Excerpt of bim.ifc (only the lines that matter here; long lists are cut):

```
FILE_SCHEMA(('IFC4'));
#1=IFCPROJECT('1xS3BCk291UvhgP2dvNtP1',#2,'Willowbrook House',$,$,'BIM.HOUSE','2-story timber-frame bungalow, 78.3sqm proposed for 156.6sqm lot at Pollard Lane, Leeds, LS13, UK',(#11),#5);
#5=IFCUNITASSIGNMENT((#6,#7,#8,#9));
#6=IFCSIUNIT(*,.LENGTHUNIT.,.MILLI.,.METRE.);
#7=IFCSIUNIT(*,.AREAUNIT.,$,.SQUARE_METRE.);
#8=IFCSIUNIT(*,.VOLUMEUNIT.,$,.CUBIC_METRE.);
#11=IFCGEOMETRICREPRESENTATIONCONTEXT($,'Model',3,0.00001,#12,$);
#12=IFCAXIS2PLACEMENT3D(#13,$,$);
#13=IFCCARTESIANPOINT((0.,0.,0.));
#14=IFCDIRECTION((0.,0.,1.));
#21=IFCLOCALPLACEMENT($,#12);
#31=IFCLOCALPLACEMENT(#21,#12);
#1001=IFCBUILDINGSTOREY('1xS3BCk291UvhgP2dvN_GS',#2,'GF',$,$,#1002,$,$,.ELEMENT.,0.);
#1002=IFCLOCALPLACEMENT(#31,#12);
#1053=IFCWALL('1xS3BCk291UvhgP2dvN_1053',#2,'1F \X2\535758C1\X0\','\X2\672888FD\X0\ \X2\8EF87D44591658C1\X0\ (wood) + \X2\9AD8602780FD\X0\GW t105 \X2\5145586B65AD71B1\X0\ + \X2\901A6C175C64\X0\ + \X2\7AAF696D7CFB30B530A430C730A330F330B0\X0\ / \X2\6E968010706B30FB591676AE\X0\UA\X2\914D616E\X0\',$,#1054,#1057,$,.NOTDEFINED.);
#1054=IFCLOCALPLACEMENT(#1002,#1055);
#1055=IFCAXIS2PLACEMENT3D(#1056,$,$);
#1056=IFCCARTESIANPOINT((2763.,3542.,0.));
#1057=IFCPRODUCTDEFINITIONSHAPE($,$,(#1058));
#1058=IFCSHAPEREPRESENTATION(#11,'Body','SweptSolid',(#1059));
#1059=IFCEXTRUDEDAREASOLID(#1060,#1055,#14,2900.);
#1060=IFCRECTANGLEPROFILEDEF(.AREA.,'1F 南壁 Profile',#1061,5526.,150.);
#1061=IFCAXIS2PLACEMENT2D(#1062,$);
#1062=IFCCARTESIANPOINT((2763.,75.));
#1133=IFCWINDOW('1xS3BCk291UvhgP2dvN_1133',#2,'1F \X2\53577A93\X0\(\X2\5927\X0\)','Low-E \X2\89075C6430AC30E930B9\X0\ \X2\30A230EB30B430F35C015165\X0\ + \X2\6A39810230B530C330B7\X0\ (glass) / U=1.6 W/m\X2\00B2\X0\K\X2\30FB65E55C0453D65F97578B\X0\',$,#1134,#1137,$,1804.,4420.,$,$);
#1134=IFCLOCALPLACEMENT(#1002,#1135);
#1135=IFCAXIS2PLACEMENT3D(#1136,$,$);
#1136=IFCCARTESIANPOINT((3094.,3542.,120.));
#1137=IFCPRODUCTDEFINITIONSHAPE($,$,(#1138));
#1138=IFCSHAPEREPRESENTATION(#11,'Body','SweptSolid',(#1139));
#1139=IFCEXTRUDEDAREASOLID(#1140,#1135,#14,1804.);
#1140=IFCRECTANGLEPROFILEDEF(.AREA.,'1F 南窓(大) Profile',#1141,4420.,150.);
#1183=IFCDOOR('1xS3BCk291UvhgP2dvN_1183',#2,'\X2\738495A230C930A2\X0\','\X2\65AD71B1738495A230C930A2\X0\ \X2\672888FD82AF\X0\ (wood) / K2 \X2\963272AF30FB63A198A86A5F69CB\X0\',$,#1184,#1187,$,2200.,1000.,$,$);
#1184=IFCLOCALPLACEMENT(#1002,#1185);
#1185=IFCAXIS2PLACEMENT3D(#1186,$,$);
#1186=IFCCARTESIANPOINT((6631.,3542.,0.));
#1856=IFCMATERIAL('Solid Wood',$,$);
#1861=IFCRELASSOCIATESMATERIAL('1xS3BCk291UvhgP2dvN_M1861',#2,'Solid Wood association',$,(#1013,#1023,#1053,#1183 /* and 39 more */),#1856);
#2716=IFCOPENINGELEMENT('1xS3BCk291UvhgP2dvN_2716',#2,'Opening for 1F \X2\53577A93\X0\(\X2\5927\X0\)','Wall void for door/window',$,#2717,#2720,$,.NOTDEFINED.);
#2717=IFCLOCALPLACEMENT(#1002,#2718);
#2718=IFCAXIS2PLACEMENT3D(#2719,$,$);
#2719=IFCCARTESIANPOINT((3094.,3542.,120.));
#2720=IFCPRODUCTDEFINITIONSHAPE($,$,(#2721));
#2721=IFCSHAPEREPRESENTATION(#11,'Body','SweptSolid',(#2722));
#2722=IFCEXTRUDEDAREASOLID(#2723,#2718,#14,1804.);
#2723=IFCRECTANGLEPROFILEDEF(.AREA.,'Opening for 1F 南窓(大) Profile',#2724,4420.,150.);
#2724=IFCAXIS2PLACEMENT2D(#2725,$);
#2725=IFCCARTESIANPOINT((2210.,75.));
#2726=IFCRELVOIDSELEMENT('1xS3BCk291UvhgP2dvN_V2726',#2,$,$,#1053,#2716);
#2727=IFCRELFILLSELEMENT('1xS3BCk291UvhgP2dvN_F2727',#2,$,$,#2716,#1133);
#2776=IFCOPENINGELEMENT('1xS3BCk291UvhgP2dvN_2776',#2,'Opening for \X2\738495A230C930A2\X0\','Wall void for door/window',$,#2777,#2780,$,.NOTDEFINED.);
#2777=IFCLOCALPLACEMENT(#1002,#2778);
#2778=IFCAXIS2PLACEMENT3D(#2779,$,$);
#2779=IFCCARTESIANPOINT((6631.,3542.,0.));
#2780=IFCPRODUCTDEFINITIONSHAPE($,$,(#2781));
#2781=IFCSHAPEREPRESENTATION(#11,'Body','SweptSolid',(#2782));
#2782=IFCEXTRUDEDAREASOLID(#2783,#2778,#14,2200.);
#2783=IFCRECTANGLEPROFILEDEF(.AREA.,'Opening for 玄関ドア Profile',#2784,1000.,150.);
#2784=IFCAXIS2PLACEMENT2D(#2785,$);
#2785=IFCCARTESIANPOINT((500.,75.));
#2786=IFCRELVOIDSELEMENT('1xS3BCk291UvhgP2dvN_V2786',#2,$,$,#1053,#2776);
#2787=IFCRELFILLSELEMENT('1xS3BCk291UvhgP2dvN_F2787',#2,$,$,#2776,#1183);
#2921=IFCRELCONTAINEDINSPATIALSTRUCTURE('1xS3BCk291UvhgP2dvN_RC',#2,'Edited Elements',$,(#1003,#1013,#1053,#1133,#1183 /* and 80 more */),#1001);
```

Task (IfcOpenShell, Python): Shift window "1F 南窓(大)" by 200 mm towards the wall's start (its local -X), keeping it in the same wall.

```python
import ifcopenshell
import ifcopenshell.api.geometry
import ifcopenshell.util.placement
import ifcopenshell.util.unit

model = ifcopenshell.open("bim.ifc")
unit_scale = ifcopenshell.util.unit.calculate_unit_scale(model)

window = model.by_guid("1xS3BCk291UvhgP2dvN_1133")
opening = window.FillsVoids[0].RelatingOpeningElement
wall = opening.VoidsElements[0].RelatingBuildingElement

wall_matrix = ifcopenshell.util.placement.get_local_placement(wall.ObjectPlacement)
shift = wall_matrix[:3, 0] * -0.2 / unit_scale
before = ifcopenshell.util.placement.get_local_placement(window.ObjectPlacement)[:3, 3].copy()

# The window is not placed relative to its opening, so move both.
for product in (opening, window):
    matrix = ifcopenshell.util.placement.get_local_placement(product.ObjectPlacement)
    matrix[:3, 3] += shift
    ifcopenshell.api.geometry.edit_object_placement(model, product=product, matrix=matrix, is_si=False)

after = ifcopenshell.util.placement.get_local_placement(window.ObjectPlacement)[:3, 3]
print("window moved by", (after - before).round(3) + 0.0)

model.write("bim-out.ifc")
```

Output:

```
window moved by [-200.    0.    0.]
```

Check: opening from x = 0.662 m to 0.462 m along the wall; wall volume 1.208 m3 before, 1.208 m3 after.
